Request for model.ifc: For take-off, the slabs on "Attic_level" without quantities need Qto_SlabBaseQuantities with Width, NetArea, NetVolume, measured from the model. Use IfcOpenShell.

First a look at what the model holds.

```python
import ifcopenshell
import ifcopenshell.util.element
import ifcopenshell.util.unit

model = ifcopenshell.open("model.ifc")
print(model.schema)
for unit_type in ("LENGTHUNIT", "AREAUNIT", "VOLUMEUNIT"):
    print(unit_type, ifcopenshell.util.unit.calculate_unit_scale(model, unit_type))
storey = next(s for s in model.by_type("IfcBuildingStorey") if s.Name == "Attic_level")
slabs = [e for e in ifcopenshell.util.element.get_decomposition(storey) if e.is_a("IfcSlab")]
for e in sorted(slabs, key=lambda e: e.id()):
    print(e.id(), e.is_a(), e.Name, list(ifcopenshell.util.element.get_psets(e, qtos_only=True)), sep=" | ")
```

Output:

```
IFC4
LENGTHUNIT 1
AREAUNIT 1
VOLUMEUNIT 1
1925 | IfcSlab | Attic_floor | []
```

```python
import ifcopenshell
import ifcopenshell.api.pset
import ifcopenshell.geom
import ifcopenshell.util.element
import ifcopenshell.util.shape
import ifcopenshell.util.unit

model = ifcopenshell.open("model.ifc")
unit_scale = ifcopenshell.util.unit.calculate_unit_scale(model)
area_scale = ifcopenshell.util.unit.calculate_unit_scale(model, "AREAUNIT")
volume_scale = ifcopenshell.util.unit.calculate_unit_scale(model, "VOLUMEUNIT")
settings = ifcopenshell.geom.settings()

storey = next(s for s in model.by_type("IfcBuildingStorey") if s.Name == "Attic_level")
slabs = [e for e in ifcopenshell.util.element.get_decomposition(storey) if e.is_a("IfcSlab")]

for e in sorted(slabs, key=lambda e: e.id()):
    if ifcopenshell.util.element.get_psets(e, qtos_only=True, should_inherit=False):
        continue
    # Geometry comes back in metres, in the element's own axes.
    shape = ifcopenshell.geom.create_shape(settings, e)
    values = {
        "Width": ifcopenshell.util.shape.get_z(shape.geometry) / unit_scale,
        "NetArea": ifcopenshell.util.shape.get_footprint_area(shape.geometry) / area_scale,
        "NetVolume": ifcopenshell.util.shape.get_volume(shape.geometry) / volume_scale,
    }
    qto = ifcopenshell.api.pset.add_qto(model, product=e, name="Qto_SlabBaseQuantities")
    ifcopenshell.api.pset.edit_qto(model, qto=qto, properties=values)
    print(e.id(), {k: round(v, 3) for k, v in values.items()})

model.write("model_updated.ifc")
```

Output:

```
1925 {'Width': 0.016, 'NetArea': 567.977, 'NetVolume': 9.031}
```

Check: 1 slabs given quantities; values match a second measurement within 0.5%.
